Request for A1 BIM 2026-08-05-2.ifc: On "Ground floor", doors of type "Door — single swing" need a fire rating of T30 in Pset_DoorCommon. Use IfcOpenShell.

First a look at what the model holds.

```python
import ifcopenshell
import ifcopenshell.util.element

model = ifcopenshell.open("A1 BIM 2026-08-05-2.ifc")
print(model.schema)
storey = next(s for s in model.by_type("IfcBuildingStorey") if s.Name == "Ground floor")
doors = [e for e in ifcopenshell.util.element.get_decomposition(storey) if e.is_a("IfcDoor")]
seen = {}
for e in doors:
    element_type = ifcopenshell.util.element.get_type(e)
    key = (element_type.Name if element_type != e and element_type else None, ifcopenshell.util.element.get_pset(e, "Pset_DoorCommon", "FireRating"))
    seen[key] = seen.get(key, 0) + 1
for (name, value), count in sorted(seen.items(), key=str):
    print(count, "x", name, "|", value)
```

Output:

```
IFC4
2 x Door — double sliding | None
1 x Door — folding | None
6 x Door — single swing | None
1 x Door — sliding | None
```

```python
import ifcopenshell
import ifcopenshell.api.pset
import ifcopenshell.util.element

model = ifcopenshell.open("A1 BIM 2026-08-05-2.ifc")

storey = next(s for s in model.by_type("IfcBuildingStorey") if s.Name == "Ground floor")
doors = [e for e in ifcopenshell.util.element.get_decomposition(storey) if e.is_a("IfcDoor")]

count = 0
for e in doors:
    element_type = ifcopenshell.util.element.get_type(e)
    if element_type in (None, e) or element_type.Name != "Door — single swing":
        continue
    # add_pset returns the element's existing set when there is one.
    pset = ifcopenshell.api.pset.add_pset(model, product=e, name="Pset_DoorCommon")
    ifcopenshell.api.pset.edit_pset(model, pset=pset, properties={"FireRating": "T30"})
    count += 1

print(count, "doors updated")

model.write("A1 BIM 2026-08-05-2_rev.ifc")
```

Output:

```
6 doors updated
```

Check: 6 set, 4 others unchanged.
